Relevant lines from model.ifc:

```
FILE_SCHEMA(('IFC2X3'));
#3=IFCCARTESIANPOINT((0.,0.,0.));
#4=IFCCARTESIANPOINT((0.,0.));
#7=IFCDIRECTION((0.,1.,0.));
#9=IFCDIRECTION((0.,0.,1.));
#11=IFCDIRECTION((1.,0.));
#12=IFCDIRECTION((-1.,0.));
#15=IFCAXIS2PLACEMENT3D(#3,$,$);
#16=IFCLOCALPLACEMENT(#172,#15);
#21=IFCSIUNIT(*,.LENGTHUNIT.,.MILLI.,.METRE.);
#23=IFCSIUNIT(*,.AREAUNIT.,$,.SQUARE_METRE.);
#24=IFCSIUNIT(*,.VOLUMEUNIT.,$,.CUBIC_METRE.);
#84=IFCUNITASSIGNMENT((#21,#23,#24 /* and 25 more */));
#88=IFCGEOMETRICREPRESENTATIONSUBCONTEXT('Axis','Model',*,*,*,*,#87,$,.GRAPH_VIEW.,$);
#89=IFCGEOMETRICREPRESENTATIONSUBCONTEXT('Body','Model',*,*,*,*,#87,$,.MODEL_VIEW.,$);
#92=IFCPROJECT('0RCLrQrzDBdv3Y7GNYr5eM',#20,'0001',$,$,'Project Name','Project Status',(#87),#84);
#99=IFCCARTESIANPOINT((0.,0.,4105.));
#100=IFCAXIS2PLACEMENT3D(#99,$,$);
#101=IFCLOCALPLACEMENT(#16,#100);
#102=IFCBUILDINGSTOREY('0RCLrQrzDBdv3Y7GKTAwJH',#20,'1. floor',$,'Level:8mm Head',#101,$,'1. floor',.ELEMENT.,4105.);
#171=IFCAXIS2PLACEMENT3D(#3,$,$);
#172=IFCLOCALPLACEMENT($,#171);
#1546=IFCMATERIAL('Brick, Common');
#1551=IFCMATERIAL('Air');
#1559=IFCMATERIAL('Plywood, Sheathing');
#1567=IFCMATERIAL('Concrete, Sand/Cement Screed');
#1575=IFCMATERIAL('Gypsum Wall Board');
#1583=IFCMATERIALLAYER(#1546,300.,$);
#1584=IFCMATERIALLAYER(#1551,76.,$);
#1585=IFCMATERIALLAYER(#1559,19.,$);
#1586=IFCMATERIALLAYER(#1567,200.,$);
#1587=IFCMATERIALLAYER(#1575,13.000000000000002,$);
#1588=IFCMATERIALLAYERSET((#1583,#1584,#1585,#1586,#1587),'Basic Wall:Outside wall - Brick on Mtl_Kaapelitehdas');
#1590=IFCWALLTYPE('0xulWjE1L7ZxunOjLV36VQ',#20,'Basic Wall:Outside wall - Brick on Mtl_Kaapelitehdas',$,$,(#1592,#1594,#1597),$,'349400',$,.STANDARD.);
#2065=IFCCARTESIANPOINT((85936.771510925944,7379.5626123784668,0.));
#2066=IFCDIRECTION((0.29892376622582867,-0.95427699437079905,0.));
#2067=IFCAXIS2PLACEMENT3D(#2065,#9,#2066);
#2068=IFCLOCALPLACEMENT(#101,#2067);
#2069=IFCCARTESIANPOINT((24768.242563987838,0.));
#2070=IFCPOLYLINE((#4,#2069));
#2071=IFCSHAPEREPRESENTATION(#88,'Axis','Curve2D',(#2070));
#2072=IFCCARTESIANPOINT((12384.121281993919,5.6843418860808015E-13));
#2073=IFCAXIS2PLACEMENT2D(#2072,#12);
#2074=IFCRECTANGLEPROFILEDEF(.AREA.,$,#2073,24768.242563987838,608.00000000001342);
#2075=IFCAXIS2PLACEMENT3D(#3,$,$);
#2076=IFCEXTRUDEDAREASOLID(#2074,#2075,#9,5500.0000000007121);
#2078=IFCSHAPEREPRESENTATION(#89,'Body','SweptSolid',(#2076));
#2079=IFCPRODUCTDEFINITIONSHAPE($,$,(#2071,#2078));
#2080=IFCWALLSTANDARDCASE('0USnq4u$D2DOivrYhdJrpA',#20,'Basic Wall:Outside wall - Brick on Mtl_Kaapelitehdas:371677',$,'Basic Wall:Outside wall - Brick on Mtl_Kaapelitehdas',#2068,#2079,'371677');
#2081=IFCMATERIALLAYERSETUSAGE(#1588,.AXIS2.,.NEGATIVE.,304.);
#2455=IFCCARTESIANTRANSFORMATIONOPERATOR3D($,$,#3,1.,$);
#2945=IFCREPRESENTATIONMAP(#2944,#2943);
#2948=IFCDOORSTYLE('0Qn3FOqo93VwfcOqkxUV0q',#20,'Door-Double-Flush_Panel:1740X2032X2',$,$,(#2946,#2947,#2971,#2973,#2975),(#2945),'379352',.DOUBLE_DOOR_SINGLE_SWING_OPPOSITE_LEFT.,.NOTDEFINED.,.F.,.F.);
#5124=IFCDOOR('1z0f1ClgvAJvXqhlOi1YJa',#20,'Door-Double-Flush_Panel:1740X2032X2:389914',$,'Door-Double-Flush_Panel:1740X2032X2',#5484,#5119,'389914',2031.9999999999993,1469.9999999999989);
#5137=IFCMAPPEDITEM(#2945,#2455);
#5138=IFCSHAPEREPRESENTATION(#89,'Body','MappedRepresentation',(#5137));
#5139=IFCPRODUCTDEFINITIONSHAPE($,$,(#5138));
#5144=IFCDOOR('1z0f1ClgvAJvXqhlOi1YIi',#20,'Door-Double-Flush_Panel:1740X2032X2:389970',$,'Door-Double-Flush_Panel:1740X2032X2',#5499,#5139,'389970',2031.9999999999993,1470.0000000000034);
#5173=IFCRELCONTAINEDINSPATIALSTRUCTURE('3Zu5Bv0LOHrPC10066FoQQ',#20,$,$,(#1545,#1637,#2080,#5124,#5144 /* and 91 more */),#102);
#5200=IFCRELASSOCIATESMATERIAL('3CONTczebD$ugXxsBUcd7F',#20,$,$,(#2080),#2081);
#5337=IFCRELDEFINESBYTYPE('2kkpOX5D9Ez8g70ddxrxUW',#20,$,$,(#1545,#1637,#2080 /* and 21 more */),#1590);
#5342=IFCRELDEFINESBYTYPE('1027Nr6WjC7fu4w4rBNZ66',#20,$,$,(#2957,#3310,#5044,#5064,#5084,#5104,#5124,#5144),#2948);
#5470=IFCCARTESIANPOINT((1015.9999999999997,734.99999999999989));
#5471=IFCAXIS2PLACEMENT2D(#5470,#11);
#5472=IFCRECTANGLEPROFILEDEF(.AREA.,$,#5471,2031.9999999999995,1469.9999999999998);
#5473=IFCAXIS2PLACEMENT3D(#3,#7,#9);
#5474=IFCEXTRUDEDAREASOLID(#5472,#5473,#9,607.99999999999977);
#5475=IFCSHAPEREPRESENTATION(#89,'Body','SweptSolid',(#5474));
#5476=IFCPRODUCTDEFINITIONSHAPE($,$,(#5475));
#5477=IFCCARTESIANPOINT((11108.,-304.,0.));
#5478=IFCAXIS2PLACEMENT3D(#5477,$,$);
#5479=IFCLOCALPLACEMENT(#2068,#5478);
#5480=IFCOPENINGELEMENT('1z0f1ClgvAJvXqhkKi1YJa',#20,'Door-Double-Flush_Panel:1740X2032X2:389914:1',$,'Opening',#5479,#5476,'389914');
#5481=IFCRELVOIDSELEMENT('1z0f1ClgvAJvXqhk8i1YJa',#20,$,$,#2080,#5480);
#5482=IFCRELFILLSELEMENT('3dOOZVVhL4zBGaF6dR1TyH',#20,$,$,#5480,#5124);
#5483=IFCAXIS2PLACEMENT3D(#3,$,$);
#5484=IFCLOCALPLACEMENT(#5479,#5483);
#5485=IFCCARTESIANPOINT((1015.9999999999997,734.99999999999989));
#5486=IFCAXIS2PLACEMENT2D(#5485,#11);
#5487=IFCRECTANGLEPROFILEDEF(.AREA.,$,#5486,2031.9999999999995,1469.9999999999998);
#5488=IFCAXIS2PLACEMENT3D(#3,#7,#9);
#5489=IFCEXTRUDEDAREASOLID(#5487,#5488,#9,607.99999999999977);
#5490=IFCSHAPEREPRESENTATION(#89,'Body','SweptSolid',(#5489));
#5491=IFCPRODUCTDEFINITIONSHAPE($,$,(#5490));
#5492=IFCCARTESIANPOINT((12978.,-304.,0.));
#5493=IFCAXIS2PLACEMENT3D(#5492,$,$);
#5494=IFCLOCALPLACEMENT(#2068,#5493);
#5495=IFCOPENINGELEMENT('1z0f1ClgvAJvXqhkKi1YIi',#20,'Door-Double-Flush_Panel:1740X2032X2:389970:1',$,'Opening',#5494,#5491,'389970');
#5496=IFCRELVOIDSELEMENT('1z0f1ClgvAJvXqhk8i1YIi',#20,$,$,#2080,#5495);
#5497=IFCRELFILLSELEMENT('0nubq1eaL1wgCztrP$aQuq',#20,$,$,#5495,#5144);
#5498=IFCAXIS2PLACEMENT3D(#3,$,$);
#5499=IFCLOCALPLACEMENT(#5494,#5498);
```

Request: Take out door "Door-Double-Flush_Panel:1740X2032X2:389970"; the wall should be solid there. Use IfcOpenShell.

```python
import ifcopenshell
import ifcopenshell.api.feature
import ifcopenshell.api.root
import ifcopenshell.geom
import ifcopenshell.util.shape

model = ifcopenshell.open("model.ifc")
settings = ifcopenshell.geom.settings()


def volume(element):
    """Net volume in cubic metres, openings subtracted."""
    shape = ifcopenshell.geom.create_shape(settings, element)
    return ifcopenshell.util.shape.get_volume(shape.geometry)


door = model.by_guid("1z0f1ClgvAJvXqhlOi1YIi")
opening = door.FillsVoids[0].RelatingOpeningElement
wall = opening.VoidsElements[0].RelatingBuildingElement
before = volume(wall)

ifcopenshell.api.root.remove_product(model, product=door)
ifcopenshell.api.feature.remove_feature(model, feature=opening)

after = volume(wall)

print(f"wall volume {before:.3f} -> {after:.3f} m3")

model.write("model-out.ifc")
```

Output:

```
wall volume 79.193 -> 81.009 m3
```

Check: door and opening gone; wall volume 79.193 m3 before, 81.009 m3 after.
